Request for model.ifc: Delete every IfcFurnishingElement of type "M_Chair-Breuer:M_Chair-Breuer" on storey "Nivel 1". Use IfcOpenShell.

First a look at what the model holds.

```python
import ifcopenshell
import ifcopenshell.util.element

model = ifcopenshell.open("model.ifc")
print(model.schema)
storey = next(s for s in model.by_type("IfcBuildingStorey") if s.Name == "Nivel 1")
furniture = [e for e in ifcopenshell.util.element.get_decomposition(storey) if e.is_a("IfcFurnishingElement")]
seen = {}
for e in furniture:
    element_type = ifcopenshell.util.element.get_type(e)
    name = element_type.Name if element_type not in (None, e) else None
    seen[name] = seen.get(name, 0) + 1
for name, count in sorted(seen.items(), key=str):
    print(count, "x", name)
```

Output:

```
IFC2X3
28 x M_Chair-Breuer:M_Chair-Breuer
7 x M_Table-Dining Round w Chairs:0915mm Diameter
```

```python
import ifcopenshell
import ifcopenshell.api.root
import ifcopenshell.util.element

model = ifcopenshell.open("model.ifc")

storey = next(s for s in model.by_type("IfcBuildingStorey") if s.Name == "Nivel 1")
furniture = [e for e in ifcopenshell.util.element.get_decomposition(storey) if e.is_a("IfcFurnishingElement")]
targets = [e for e in furniture if (t := ifcopenshell.util.element.get_type(e)) not in (None, e) and t.Name == "M_Chair-Breuer:M_Chair-Breuer"]

for e in targets:
    ifcopenshell.api.root.remove_product(model, product=e)
print(len(targets), "removed")

model.write("model_updated.ifc")
```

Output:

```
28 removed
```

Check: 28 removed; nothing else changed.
